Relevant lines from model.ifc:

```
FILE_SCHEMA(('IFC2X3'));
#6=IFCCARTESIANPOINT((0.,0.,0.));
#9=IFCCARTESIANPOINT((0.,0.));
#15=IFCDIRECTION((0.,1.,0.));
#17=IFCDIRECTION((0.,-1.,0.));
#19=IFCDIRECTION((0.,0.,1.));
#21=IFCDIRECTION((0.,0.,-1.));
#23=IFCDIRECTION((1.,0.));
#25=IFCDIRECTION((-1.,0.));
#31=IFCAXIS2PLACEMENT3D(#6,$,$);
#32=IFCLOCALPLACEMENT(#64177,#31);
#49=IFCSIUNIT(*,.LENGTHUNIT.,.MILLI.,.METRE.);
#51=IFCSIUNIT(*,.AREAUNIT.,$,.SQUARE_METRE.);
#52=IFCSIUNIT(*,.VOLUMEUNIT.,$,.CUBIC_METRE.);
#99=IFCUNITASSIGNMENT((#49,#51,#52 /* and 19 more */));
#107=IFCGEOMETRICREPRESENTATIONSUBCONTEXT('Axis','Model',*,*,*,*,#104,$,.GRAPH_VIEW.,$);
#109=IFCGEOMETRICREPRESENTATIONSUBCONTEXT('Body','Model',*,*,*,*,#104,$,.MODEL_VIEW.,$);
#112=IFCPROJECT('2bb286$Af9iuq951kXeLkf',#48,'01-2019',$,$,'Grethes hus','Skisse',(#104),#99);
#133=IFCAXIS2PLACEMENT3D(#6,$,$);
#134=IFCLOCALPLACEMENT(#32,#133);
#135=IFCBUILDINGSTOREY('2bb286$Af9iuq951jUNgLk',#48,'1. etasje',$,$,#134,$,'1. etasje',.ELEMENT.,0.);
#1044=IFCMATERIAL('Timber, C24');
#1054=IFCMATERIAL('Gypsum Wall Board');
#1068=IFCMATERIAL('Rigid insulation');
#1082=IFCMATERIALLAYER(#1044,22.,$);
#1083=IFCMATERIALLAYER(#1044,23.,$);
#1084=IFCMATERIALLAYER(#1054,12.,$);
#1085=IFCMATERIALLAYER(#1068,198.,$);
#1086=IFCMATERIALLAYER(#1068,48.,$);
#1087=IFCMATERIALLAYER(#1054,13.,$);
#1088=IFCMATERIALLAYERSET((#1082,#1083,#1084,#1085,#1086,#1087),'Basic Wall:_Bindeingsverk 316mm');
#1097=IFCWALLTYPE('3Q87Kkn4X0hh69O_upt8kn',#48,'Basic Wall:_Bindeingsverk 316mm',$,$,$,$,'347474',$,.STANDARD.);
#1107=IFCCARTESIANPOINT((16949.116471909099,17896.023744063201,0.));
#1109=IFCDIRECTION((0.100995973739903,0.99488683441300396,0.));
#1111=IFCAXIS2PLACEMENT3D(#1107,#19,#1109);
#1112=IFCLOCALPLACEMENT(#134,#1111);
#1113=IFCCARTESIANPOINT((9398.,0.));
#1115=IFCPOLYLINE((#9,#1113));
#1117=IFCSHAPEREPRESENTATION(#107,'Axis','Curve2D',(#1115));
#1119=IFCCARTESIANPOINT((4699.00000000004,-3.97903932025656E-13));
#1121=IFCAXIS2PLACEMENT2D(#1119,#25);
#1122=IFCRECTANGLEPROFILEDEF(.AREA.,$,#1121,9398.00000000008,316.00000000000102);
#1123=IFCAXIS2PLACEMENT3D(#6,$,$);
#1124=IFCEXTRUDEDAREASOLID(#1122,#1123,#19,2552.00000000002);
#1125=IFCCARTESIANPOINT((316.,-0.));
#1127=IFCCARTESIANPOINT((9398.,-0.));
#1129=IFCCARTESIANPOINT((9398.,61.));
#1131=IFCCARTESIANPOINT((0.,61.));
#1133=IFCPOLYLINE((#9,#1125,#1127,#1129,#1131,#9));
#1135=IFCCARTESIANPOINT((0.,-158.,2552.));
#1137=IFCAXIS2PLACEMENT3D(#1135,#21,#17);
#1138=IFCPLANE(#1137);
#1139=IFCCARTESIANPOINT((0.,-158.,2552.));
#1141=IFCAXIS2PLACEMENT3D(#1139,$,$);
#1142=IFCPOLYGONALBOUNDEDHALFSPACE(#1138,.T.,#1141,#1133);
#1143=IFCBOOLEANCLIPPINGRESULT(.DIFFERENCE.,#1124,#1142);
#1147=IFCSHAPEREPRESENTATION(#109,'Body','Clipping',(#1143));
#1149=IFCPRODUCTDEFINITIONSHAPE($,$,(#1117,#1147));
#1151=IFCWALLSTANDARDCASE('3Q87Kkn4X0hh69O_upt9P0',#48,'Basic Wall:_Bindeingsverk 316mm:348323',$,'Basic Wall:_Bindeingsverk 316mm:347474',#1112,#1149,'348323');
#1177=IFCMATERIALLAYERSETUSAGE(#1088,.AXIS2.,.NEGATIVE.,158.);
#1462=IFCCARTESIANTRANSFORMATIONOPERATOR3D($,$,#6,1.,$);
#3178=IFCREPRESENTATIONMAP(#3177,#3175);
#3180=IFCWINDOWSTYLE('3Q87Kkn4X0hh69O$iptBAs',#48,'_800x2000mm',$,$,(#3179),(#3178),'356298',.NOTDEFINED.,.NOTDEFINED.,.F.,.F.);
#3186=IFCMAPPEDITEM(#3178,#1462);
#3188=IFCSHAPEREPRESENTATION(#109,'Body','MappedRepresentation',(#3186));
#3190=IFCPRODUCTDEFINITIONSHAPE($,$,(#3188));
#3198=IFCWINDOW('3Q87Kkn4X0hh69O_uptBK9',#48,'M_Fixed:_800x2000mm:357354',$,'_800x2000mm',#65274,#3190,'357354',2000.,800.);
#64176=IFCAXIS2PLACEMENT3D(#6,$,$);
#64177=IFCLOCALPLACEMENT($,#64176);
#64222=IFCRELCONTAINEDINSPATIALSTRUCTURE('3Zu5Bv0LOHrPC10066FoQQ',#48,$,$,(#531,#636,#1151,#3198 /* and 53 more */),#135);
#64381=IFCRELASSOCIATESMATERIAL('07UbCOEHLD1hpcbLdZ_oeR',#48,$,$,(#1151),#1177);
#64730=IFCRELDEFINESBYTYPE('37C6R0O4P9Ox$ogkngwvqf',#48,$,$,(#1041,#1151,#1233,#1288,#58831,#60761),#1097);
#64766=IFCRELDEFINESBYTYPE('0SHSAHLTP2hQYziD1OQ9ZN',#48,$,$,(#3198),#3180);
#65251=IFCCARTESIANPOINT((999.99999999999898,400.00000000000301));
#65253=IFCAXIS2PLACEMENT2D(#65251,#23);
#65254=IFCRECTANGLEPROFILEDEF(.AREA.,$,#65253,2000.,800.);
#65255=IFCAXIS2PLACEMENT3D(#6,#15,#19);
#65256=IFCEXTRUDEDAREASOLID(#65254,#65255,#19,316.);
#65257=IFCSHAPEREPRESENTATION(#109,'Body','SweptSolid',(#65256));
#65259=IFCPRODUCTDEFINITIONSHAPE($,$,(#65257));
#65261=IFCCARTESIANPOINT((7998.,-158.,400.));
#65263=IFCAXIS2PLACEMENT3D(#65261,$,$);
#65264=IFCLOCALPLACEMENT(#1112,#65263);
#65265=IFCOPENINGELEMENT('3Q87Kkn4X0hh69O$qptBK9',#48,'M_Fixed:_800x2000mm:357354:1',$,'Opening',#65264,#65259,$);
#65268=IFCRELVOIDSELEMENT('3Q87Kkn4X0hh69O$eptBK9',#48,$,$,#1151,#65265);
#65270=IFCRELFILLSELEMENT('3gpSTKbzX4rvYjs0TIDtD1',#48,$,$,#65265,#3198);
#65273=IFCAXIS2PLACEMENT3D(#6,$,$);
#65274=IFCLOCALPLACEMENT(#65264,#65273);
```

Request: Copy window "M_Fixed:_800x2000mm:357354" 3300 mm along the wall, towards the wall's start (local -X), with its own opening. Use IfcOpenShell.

```python
import ifcopenshell
import ifcopenshell.api.feature
import ifcopenshell.api.geometry
import ifcopenshell.api.root
import ifcopenshell.geom
import ifcopenshell.util.element
import ifcopenshell.util.placement
import ifcopenshell.util.shape
import ifcopenshell.util.unit

model = ifcopenshell.open("model.ifc")
unit_scale = ifcopenshell.util.unit.calculate_unit_scale(model)
settings = ifcopenshell.geom.settings()


def volume(element):
    """Net volume in cubic metres, openings subtracted."""
    shape = ifcopenshell.geom.create_shape(settings, element)
    return ifcopenshell.util.shape.get_volume(shape.geometry)


def reuse_history(source, copy):
    """copy_class also copies each property set's owner history, people and application; keep the originals."""
    for rel in copy.IsDefinedBy:
        if rel.is_a("IfcRelDefinesByProperties") and (history := rel.RelatingPropertyDefinition.OwnerHistory):
            rel.RelatingPropertyDefinition.OwnerHistory = source.OwnerHistory
            ifcopenshell.util.element.remove_deep2(model, history)


window = model.by_guid("3Q87Kkn4X0hh69O_uptBK9")
opening = window.FillsVoids[0].RelatingOpeningElement
wall = opening.VoidsElements[0].RelatingBuildingElement
before = volume(wall)
shift = ifcopenshell.util.placement.get_local_placement(wall.ObjectPlacement)[:3, 0] * -3.3 / unit_scale

# copy_class copies the void relationship, type, container and properties, but no geometry.
new_opening = ifcopenshell.api.root.copy_class(model, product=opening)
new_opening.Representation = ifcopenshell.util.element.copy_deep(
    model, opening.Representation, exclude=["IfcGeometricRepresentationContext", "IfcRepresentationMap"]
)
new_opening.Name = "M_Fixed:_800x2000mm"
new_window = ifcopenshell.api.root.copy_class(model, product=window)
new_window.Representation = ifcopenshell.util.element.copy_deep(
    model, window.Representation, exclude=["IfcGeometricRepresentationContext", "IfcRepresentationMap"]
)
new_window.Name = "M_Fixed:_800x2000mm"
new_window.Tag = None
reuse_history(window, new_window)
fills = ifcopenshell.api.feature.add_filling(model, opening=new_opening, element=new_window)
fills.OwnerHistory = new_window.OwnerHistory  # required in IFC2X3

for old, new in ((opening, new_opening), (window, new_window)):
    matrix = ifcopenshell.util.placement.get_local_placement(old.ObjectPlacement)
    matrix[:3, 3] += shift
    ifcopenshell.api.geometry.edit_object_placement(model, product=new, matrix=matrix, is_si=False)

after = volume(wall)

print(f"wall volume {before:.3f} -> {after:.3f} m3")

model.write("model_edited.ifc")
```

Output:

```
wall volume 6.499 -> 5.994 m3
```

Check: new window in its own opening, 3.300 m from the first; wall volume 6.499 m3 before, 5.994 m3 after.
